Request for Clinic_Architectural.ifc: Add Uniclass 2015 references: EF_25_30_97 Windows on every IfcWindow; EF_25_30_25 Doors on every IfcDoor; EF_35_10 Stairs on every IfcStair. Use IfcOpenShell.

First a look at what the model holds.

```python
import ifcopenshell

model = ifcopenshell.open("Clinic_Architectural.ifc")
print(model.schema)
print("classifications:", [c.Name for c in model.by_type("IfcClassification")])
for ifc_class in ("IfcDoor", "IfcRoof", "IfcStair", "IfcWall", "IfcWindow"):
    print(ifc_class, len(model.by_type(ifc_class)))
```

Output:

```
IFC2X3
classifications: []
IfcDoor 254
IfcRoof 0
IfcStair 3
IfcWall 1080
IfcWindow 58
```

```python
import ifcopenshell
import ifcopenshell.api.classification

model = ifcopenshell.open("Clinic_Architectural.ifc")

# IFC2X3 requires Source and Edition and has no link from the project to the system.
system = model.create_entity("IfcClassification", Source="NBS", Edition="2015", Name="Uniclass 2015")

codes = {
    "IfcWindow": ("EF_25_30_97", "Windows"),
    "IfcDoor": ("EF_25_30_25", "Doors"),
    "IfcStair": ("EF_35_10", "Stairs"),
}
for ifc_class, (code, name) in codes.items():
    products = model.by_type(ifc_class)
    ifcopenshell.api.classification.add_reference(
        model, products=products, classification=system, identification=code, name=name
    )
    print(code, len(products))

model.write("Clinic_Architectural_rev.ifc")
```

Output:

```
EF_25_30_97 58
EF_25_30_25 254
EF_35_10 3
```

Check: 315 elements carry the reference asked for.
